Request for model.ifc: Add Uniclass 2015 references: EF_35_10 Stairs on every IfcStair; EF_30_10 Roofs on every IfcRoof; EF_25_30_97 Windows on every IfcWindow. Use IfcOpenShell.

First a look at what the model holds.

```python
import ifcopenshell

model = ifcopenshell.open("model.ifc")
print(model.schema)
print("classifications:", [c.Name for c in model.by_type("IfcClassification")])
for ifc_class in ("IfcDoor", "IfcRoof", "IfcStair", "IfcWall", "IfcWindow"):
    print(ifc_class, len(model.by_type(ifc_class)))
```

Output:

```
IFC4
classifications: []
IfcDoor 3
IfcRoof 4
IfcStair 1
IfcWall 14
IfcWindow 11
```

```python
import ifcopenshell
import ifcopenshell.api.classification

model = ifcopenshell.open("model.ifc")

system = ifcopenshell.api.classification.add_classification(model, classification="Uniclass 2015")

codes = {
    "IfcStair": ("EF_35_10", "Stairs"),
    "IfcRoof": ("EF_30_10", "Roofs"),
    "IfcWindow": ("EF_25_30_97", "Windows"),
}
for ifc_class, (code, name) in codes.items():
    products = model.by_type(ifc_class)
    ifcopenshell.api.classification.add_reference(
        model, products=products, classification=system, identification=code, name=name
    )
    print(code, len(products))

model.write("model_v2.ifc")
```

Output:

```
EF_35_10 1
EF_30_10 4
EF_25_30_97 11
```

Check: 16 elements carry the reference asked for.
